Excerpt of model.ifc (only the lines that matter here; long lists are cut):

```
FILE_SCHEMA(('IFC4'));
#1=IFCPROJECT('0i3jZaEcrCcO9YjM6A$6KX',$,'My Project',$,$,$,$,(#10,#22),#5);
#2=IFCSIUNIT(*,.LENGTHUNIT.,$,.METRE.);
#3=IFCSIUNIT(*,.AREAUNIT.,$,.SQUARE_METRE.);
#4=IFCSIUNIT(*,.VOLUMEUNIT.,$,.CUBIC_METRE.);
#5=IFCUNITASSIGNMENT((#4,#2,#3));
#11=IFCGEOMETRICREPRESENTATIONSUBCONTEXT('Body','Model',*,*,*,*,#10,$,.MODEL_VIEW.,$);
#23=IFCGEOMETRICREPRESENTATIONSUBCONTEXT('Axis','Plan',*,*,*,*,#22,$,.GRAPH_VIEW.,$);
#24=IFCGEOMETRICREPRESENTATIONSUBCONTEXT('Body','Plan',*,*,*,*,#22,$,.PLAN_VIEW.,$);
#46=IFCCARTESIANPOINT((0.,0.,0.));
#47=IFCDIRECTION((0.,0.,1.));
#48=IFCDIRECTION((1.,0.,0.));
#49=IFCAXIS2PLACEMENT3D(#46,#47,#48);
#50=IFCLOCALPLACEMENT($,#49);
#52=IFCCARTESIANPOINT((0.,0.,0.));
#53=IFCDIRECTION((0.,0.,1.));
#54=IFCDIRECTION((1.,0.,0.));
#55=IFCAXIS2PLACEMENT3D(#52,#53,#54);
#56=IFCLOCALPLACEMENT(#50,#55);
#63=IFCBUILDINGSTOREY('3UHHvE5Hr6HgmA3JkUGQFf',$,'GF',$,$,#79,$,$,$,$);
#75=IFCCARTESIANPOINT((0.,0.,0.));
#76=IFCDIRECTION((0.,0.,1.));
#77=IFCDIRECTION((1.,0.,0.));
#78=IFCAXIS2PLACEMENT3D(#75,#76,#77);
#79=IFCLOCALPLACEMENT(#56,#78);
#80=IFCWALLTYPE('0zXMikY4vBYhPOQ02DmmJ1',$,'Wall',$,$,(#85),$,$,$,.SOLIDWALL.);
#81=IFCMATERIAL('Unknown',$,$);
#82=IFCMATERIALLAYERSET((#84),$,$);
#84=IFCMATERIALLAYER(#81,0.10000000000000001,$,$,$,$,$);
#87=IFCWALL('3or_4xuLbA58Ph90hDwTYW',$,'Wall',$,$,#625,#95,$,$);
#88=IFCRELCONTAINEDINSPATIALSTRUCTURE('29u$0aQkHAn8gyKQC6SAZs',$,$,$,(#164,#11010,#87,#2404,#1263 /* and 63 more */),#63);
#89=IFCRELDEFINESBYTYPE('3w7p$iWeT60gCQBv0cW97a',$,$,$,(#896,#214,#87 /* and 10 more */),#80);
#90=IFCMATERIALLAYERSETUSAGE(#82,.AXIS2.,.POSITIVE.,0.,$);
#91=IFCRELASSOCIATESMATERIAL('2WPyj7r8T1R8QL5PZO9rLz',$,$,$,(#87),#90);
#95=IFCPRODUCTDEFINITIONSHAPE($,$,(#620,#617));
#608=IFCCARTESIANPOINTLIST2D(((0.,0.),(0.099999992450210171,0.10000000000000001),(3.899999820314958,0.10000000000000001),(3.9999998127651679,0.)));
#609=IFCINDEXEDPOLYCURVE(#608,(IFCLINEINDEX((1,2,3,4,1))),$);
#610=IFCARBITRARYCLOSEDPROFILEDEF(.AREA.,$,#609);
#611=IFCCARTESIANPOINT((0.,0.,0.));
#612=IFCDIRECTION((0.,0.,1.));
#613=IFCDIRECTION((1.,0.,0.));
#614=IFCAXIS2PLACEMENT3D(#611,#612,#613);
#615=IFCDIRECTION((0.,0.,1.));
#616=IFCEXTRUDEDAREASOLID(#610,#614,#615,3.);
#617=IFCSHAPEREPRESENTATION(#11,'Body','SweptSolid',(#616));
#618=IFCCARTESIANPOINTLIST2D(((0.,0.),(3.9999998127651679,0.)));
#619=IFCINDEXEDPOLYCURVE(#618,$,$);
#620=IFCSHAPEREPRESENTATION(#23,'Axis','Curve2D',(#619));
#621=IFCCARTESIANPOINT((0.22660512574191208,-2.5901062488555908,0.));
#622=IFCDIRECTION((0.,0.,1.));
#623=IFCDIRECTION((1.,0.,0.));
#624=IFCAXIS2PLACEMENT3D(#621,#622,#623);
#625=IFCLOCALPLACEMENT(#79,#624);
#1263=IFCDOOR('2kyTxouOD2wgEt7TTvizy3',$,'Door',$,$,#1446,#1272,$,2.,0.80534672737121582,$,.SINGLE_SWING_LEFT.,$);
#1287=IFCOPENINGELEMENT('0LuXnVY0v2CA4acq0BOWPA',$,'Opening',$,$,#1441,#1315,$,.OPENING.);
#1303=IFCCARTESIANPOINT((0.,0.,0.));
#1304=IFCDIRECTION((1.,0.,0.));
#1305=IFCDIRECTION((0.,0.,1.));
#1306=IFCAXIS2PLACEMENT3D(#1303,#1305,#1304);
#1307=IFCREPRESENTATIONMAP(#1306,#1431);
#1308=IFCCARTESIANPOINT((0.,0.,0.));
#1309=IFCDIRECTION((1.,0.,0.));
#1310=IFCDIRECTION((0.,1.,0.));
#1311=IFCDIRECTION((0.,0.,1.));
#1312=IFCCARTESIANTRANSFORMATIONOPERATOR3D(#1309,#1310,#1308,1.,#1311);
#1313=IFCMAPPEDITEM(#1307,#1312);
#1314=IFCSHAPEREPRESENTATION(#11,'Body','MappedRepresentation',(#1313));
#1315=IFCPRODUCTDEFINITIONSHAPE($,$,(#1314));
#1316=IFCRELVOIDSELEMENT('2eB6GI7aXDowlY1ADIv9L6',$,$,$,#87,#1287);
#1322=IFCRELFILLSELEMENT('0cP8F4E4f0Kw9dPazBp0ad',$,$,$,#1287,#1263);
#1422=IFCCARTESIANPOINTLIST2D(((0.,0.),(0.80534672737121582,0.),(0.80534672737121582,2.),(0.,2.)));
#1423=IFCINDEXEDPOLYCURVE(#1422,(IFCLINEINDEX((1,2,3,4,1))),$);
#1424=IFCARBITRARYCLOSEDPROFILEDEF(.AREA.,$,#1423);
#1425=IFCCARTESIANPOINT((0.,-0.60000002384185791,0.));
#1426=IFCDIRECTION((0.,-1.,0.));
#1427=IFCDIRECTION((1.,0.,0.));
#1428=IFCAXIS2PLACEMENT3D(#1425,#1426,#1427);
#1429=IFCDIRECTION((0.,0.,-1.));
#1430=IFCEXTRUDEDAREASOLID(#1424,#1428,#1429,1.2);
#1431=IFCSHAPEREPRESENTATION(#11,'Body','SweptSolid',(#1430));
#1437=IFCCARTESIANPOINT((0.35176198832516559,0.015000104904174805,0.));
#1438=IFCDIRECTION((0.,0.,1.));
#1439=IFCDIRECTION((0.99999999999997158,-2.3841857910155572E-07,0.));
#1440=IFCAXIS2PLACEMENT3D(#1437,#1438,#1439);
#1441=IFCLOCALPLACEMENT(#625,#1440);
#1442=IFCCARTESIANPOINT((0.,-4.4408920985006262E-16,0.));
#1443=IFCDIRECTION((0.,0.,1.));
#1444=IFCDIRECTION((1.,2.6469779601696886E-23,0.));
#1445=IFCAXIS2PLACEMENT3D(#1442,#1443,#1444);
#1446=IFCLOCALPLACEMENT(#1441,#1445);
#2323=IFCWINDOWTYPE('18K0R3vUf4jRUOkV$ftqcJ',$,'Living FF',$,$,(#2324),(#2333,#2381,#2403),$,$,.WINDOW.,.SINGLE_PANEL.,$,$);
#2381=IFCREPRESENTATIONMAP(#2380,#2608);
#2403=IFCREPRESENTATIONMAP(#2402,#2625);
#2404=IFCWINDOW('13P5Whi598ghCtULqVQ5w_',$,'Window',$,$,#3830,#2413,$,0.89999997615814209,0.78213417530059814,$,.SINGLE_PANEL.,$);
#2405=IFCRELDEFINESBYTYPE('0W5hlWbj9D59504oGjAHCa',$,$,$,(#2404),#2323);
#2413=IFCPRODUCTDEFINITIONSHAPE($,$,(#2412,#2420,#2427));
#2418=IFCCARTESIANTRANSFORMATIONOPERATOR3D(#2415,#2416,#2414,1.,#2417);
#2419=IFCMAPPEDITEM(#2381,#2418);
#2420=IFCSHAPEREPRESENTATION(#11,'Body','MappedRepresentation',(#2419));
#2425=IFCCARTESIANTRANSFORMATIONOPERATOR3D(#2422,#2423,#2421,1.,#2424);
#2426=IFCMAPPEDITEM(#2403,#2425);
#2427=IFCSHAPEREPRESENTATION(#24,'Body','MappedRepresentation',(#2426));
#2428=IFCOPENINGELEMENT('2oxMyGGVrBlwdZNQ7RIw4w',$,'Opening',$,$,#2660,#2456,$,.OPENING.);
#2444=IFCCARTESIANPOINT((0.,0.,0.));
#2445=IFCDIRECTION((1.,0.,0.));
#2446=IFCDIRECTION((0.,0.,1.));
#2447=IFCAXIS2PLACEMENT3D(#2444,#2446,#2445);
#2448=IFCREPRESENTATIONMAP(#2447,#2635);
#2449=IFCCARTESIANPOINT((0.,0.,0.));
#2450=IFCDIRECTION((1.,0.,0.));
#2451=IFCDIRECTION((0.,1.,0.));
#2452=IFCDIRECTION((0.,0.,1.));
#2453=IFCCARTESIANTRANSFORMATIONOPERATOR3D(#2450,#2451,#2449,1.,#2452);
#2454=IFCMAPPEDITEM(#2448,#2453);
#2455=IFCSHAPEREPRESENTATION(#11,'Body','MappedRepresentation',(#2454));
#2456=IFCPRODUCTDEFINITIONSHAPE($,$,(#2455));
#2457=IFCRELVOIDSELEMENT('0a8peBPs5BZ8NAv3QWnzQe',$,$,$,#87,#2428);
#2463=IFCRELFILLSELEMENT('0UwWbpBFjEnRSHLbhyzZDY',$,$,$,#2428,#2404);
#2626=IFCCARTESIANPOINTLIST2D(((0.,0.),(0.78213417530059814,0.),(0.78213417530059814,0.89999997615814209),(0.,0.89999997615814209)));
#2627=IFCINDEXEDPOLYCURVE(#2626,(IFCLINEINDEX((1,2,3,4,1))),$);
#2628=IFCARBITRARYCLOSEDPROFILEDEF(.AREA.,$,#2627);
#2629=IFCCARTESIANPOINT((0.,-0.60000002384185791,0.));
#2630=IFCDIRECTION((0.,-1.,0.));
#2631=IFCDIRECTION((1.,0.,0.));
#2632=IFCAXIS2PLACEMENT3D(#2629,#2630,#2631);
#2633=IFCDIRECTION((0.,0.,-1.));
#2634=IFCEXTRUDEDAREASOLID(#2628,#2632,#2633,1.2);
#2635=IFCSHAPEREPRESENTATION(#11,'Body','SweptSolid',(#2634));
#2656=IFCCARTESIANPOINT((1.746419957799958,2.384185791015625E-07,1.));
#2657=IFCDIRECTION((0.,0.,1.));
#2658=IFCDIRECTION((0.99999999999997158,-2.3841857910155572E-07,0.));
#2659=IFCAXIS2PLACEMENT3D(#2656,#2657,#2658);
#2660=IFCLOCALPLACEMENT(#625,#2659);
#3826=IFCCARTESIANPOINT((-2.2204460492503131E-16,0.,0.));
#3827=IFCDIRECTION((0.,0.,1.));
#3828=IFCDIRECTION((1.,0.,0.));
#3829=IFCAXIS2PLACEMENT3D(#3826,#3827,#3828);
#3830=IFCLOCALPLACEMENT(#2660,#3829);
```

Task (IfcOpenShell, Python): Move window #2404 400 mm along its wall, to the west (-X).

```python
import ifcopenshell
import ifcopenshell.api.geometry
import ifcopenshell.util.placement

model = ifcopenshell.open("model.ifc")

window = model.by_id(2404)
opening = window.FillsVoids[0].RelatingOpeningElement
wall = opening.VoidsElements[0].RelatingBuildingElement

wall_matrix = ifcopenshell.util.placement.get_local_placement(wall.ObjectPlacement)
shift = wall_matrix[:3, 0] * -0.4
before = ifcopenshell.util.placement.get_local_placement(window.ObjectPlacement)[:3, 3].copy()

# The window is placed relative to its opening, so it follows when the opening moves.
matrix = ifcopenshell.util.placement.get_local_placement(opening.ObjectPlacement)
matrix[:3, 3] += shift
ifcopenshell.api.geometry.edit_object_placement(
    model, product=opening, matrix=matrix, is_si=False, should_transform_children=True
)

after = ifcopenshell.util.placement.get_local_placement(window.ObjectPlacement)[:3, 3]
print("window moved by", (after - before).round(3) + 0.0)

model.write("model_edited.ifc")
```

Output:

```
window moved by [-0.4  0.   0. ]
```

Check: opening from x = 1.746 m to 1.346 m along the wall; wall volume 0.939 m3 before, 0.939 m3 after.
